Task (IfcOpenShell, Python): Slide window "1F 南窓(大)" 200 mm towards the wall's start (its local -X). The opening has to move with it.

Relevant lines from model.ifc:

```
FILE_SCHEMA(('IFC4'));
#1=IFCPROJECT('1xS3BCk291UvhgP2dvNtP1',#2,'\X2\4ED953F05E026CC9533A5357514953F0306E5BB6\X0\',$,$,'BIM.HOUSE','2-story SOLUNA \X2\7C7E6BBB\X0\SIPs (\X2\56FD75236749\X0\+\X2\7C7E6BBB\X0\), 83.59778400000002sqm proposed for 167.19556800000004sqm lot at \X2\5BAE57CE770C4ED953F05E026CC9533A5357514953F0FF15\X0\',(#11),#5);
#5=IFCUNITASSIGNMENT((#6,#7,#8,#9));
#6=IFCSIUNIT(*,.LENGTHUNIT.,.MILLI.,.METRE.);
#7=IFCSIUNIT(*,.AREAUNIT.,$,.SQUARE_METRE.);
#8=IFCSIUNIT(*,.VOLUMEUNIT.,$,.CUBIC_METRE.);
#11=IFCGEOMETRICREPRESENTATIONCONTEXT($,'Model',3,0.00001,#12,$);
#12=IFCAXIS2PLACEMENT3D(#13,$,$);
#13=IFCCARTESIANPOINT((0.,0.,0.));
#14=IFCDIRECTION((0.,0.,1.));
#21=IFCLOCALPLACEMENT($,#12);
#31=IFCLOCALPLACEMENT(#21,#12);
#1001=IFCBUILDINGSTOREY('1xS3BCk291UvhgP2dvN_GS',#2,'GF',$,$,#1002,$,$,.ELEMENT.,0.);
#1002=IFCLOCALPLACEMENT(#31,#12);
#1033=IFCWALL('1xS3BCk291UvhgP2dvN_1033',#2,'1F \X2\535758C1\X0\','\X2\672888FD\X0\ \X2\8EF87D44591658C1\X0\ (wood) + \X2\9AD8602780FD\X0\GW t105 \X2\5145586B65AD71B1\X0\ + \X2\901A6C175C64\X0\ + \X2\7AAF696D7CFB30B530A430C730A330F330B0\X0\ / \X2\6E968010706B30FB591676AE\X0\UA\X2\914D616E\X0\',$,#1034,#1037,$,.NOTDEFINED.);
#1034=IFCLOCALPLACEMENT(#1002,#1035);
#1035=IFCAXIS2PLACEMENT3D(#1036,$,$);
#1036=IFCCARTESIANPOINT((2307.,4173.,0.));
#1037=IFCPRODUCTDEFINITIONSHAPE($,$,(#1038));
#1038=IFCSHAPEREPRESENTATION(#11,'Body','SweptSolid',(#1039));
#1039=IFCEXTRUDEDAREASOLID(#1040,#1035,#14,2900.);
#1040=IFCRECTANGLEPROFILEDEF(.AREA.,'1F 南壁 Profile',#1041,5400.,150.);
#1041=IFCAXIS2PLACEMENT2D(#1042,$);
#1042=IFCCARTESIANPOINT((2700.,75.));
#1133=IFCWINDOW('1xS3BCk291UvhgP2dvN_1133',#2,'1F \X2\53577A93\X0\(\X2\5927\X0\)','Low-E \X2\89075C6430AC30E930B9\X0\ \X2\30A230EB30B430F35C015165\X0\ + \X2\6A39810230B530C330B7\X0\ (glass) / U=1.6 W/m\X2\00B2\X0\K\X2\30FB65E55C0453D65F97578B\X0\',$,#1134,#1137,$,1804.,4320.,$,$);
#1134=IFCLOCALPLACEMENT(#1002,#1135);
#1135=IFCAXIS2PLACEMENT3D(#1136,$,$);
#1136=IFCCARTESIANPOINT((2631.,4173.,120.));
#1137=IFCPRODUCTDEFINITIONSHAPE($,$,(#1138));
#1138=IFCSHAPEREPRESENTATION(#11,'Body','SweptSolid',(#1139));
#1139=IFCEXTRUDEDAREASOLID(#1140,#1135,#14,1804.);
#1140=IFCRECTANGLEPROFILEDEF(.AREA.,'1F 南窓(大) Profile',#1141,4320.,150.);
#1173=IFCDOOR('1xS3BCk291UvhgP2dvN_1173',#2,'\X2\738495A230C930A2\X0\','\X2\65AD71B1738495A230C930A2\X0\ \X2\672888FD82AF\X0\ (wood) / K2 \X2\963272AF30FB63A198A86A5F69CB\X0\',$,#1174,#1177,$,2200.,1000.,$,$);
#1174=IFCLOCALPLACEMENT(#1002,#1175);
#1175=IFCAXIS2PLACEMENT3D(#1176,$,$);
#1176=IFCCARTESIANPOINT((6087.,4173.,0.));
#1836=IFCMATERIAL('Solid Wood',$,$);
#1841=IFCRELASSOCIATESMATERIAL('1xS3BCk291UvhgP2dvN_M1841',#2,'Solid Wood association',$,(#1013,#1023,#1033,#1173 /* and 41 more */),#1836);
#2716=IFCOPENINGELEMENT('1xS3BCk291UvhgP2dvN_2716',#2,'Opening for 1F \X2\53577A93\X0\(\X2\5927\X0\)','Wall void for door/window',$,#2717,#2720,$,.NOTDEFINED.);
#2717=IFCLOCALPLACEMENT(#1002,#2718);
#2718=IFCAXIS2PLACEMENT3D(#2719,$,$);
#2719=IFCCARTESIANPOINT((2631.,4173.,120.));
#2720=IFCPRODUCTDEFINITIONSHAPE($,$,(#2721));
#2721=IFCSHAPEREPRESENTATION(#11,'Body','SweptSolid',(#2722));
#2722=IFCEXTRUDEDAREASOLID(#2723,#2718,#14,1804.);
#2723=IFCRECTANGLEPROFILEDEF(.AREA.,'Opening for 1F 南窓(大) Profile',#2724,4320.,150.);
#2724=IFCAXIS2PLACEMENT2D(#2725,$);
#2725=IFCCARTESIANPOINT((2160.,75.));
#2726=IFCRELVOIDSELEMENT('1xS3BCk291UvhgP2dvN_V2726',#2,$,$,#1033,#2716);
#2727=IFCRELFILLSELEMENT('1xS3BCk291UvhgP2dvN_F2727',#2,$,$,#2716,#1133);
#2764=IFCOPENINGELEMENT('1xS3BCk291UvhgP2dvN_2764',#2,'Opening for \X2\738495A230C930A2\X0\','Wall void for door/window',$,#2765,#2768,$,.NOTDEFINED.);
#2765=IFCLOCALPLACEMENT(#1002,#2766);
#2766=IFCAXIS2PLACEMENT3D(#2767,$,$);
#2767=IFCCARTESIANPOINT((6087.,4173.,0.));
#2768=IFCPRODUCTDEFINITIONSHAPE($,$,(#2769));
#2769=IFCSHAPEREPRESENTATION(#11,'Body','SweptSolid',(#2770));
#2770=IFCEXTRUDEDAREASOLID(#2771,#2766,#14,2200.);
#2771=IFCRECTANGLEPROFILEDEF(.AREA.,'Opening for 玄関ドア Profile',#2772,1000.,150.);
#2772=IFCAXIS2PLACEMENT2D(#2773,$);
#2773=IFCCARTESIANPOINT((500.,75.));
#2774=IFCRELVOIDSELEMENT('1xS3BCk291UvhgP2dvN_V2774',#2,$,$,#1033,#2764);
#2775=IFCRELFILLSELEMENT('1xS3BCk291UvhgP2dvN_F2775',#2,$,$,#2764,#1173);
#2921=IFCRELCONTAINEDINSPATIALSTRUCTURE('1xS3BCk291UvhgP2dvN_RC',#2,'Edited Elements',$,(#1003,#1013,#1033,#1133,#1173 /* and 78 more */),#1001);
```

```python
import ifcopenshell
import ifcopenshell.api.geometry
import ifcopenshell.util.placement

model = ifcopenshell.open("model.ifc")

window = model.by_id(1133)
opening = window.FillsVoids[0].RelatingOpeningElement
wall = opening.VoidsElements[0].RelatingBuildingElement

wall_matrix = ifcopenshell.util.placement.get_local_placement(wall.ObjectPlacement)
shift = wall_matrix[:3, 0] * -200.0
before = ifcopenshell.util.placement.get_local_placement(window.ObjectPlacement)[:3, 3].copy()

# The window is not placed relative to its opening, so move both.
for product in (opening, window):
    matrix = ifcopenshell.util.placement.get_local_placement(product.ObjectPlacement)
    matrix[:3, 3] += shift
    ifcopenshell.api.geometry.edit_object_placement(model, product=product, matrix=matrix, is_si=False)

after = ifcopenshell.util.placement.get_local_placement(window.ObjectPlacement)[:3, 3]
print("window moved by", (after - before).round(3) + 0.0)

model.write("model-out.ifc")
```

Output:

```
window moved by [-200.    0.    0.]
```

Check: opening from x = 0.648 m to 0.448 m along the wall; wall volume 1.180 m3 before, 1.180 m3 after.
